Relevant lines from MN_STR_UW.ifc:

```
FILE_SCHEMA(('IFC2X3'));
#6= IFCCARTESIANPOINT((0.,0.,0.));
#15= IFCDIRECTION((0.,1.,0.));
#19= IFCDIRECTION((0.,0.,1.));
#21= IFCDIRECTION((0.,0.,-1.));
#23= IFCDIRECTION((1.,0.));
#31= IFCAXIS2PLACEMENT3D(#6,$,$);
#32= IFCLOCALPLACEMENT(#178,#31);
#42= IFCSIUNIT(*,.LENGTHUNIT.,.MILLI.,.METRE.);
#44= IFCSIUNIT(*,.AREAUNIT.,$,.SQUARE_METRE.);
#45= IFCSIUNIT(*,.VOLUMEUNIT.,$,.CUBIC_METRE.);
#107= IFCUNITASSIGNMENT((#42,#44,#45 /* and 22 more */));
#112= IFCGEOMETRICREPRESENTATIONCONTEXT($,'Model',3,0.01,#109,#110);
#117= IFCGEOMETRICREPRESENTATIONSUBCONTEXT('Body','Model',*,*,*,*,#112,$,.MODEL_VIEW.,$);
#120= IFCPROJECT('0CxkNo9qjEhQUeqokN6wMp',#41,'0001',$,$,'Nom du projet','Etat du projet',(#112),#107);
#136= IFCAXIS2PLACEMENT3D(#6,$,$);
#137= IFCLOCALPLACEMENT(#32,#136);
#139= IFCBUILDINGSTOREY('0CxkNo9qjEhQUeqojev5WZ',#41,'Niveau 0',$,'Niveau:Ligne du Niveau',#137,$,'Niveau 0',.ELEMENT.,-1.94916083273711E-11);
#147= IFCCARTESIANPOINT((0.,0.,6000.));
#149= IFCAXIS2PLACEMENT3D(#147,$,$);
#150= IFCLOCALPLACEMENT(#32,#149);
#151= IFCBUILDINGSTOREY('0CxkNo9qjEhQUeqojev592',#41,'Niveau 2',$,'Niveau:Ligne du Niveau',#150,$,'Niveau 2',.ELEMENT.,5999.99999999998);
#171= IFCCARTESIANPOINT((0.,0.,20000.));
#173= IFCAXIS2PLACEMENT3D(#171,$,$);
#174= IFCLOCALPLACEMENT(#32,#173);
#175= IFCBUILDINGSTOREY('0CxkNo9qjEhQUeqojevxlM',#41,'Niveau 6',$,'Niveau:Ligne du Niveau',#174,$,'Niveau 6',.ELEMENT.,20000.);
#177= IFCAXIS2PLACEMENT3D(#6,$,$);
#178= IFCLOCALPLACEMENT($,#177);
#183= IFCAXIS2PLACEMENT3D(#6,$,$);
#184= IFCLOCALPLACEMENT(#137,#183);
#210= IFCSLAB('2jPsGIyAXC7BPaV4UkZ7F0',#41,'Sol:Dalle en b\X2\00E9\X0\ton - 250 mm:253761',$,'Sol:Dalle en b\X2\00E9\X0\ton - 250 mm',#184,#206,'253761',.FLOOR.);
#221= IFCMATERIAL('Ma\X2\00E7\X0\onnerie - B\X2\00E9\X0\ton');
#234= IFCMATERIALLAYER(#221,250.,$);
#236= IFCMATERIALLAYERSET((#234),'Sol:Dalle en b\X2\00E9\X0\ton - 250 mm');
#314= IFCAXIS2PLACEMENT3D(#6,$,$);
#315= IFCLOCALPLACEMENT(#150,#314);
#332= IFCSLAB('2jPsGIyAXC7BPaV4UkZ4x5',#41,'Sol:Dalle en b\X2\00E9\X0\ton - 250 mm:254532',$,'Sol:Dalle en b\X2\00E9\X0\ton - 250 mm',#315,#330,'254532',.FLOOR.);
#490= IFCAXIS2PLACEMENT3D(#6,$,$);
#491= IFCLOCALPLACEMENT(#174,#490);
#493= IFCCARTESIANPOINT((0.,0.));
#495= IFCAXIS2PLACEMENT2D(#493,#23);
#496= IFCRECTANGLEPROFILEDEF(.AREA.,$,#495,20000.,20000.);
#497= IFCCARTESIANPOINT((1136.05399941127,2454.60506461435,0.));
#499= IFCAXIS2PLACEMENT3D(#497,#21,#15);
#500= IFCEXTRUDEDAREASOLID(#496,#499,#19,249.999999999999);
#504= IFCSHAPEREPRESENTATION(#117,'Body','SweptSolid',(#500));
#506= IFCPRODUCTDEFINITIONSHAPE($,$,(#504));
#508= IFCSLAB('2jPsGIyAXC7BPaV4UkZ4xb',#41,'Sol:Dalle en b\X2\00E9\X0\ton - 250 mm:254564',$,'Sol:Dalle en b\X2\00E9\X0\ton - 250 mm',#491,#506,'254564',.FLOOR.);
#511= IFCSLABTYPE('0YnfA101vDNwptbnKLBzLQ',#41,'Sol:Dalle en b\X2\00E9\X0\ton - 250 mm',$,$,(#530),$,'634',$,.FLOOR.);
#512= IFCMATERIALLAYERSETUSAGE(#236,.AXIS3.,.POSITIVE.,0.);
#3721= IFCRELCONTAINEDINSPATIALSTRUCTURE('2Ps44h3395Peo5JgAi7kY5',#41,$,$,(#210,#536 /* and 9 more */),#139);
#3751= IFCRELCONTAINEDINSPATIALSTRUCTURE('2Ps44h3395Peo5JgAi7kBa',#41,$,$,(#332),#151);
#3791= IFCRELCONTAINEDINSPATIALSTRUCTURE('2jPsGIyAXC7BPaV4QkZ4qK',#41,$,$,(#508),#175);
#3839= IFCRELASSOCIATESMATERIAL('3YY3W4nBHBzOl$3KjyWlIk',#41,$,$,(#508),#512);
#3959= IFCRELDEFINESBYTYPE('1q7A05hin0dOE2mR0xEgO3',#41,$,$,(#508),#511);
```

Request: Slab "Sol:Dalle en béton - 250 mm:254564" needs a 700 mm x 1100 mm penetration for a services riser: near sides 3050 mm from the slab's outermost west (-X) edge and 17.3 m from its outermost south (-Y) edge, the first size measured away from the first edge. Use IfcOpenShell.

```python
import numpy as np
import ifcopenshell
import ifcopenshell.api.feature
import ifcopenshell.api.geometry
import ifcopenshell.api.root
import ifcopenshell.geom
import ifcopenshell.util.placement
import ifcopenshell.util.representation
import ifcopenshell.util.shape
import ifcopenshell.util.unit

model = ifcopenshell.open("MN_STR_UW.ifc")
unit_scale = ifcopenshell.util.unit.calculate_unit_scale(model)
settings = ifcopenshell.geom.settings()


def volume(element):
    """Net volume in cubic metres, openings subtracted."""
    shape = ifcopenshell.geom.create_shape(settings, element)
    return ifcopenshell.util.shape.get_volume(shape.geometry)


slab = model.by_guid("2jPsGIyAXC7BPaV4UkZ4xb")
before = volume(slab)

# Extent in the slab's own axes, in metres. The edges named are its -X and -Y sides.
slab_shape = ifcopenshell.geom.create_shape(settings, slab)
vertices = ifcopenshell.util.shape.get_vertices(slab_shape.geometry)
x_min, y_min, bottom = vertices.min(axis=0)
top = vertices[:, 2].max()

opening = ifcopenshell.api.root.create_entity(model, ifc_class="IfcOpeningElement", name="Services riser opening")
context = ifcopenshell.util.representation.get_context(model, "Model", "Body", "MODEL_VIEW")
width, depth = 0.7, 1.1
outline = [(0.0, 0.0), (width, 0.0), (width, depth), (0.0, depth), (0.0, 0.0)]
# Overshoot both faces by 50 mm so the cut is clean.
shape = ifcopenshell.api.geometry.add_slab_representation(
    model, context=context, depth=top - bottom + 0.1, polyline=outline
)
ifcopenshell.api.geometry.assign_representation(model, product=opening, representation=shape)

matrix = ifcopenshell.util.placement.get_local_placement(slab.ObjectPlacement)
matrix[:, 3] = matrix @ np.append(np.array([x_min + 3.05, y_min + 17.3, bottom - 0.05]) / unit_scale, 1.0)
ifcopenshell.api.geometry.edit_object_placement(model, product=opening, matrix=matrix, is_si=False)
ifcopenshell.api.feature.add_feature(model, feature=opening, element=slab)

after = volume(slab)

print(f"slab volume {before:.3f} -> {after:.3f} m3")

model.write("MN_STR_UW_edited.ifc")
```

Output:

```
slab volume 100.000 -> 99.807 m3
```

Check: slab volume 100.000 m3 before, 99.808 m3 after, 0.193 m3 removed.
